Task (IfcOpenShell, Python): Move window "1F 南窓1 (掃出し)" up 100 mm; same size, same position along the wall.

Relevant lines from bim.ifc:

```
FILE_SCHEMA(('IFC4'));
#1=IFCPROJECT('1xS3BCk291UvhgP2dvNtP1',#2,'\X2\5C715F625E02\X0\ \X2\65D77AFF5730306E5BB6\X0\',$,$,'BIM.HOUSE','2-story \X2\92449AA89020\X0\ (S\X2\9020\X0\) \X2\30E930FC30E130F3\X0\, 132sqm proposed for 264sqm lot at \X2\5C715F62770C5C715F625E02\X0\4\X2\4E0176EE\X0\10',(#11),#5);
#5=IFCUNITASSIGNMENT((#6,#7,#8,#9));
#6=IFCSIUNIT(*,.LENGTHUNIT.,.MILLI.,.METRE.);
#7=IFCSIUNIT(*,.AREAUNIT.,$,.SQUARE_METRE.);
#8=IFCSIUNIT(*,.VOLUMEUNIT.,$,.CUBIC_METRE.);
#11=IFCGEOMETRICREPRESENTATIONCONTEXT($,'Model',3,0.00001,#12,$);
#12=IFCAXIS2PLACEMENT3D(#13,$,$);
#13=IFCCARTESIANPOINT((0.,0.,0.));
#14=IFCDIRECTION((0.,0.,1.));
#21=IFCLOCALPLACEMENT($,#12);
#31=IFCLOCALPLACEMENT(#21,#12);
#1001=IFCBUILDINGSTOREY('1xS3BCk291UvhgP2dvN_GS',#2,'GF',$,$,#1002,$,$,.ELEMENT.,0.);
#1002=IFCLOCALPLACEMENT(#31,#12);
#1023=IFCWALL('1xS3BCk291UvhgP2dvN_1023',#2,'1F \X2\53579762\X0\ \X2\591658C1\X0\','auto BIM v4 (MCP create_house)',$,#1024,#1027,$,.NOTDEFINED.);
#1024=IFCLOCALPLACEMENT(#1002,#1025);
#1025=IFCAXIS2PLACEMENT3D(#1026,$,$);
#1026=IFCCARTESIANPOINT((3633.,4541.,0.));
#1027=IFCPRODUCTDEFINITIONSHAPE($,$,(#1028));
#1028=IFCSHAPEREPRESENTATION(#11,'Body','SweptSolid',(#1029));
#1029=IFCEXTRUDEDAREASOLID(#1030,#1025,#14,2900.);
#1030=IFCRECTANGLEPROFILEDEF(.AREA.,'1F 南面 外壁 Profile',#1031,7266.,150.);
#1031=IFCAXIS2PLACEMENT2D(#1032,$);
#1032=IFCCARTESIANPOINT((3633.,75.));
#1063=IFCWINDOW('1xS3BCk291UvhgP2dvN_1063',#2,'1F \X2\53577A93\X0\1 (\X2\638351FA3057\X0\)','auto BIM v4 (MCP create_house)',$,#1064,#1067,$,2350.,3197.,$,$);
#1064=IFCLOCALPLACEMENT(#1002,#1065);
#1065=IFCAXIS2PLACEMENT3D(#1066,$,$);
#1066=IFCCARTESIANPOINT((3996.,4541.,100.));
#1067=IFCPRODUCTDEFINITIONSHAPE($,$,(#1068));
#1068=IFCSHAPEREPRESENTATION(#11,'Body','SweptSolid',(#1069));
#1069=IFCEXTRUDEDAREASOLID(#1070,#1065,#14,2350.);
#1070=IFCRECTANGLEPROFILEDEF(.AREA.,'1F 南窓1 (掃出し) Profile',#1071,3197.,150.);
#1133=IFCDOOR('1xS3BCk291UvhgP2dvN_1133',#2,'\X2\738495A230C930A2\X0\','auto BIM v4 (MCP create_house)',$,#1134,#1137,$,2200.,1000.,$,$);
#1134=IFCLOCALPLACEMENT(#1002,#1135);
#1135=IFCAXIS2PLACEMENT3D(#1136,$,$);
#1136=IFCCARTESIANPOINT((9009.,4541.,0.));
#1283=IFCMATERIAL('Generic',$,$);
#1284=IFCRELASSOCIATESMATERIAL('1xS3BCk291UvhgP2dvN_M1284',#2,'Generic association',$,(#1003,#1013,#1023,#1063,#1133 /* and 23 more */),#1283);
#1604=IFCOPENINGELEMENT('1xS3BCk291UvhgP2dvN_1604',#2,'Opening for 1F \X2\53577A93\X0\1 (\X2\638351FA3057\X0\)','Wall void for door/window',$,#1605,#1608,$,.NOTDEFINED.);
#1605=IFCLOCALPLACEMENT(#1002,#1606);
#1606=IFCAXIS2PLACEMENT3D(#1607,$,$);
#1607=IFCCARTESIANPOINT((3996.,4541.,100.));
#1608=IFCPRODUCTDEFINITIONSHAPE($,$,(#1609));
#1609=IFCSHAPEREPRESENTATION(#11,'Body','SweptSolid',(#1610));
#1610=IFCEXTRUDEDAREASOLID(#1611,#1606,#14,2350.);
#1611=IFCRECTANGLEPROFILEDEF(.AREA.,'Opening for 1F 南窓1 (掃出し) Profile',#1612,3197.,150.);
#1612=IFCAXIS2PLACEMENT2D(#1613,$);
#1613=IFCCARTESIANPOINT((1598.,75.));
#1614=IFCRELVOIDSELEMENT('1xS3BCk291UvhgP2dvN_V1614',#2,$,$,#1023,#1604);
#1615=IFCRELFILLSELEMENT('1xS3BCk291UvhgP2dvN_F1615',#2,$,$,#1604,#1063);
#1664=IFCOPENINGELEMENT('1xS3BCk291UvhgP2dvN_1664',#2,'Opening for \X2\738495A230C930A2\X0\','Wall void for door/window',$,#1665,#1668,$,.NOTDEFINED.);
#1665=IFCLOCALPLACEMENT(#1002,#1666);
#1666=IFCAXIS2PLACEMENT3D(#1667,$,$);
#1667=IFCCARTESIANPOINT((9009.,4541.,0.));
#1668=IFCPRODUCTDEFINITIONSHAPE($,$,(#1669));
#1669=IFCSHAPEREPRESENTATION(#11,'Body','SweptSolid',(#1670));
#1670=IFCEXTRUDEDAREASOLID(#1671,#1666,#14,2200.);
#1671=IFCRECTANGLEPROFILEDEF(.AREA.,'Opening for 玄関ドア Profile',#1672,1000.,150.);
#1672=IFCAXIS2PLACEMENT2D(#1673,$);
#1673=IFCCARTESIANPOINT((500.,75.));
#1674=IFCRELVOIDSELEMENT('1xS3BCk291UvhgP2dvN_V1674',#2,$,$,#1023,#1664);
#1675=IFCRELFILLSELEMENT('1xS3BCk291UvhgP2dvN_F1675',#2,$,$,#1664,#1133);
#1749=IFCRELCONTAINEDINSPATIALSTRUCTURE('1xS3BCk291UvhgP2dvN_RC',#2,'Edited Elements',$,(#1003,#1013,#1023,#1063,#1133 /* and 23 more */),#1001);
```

```python
import numpy as np
import ifcopenshell
import ifcopenshell.api.geometry
import ifcopenshell.util.placement
import ifcopenshell.util.unit

model = ifcopenshell.open("bim.ifc")
unit_scale = ifcopenshell.util.unit.calculate_unit_scale(model)

window = model.by_guid("1xS3BCk291UvhgP2dvN_1063")
opening = window.FillsVoids[0].RelatingOpeningElement
dz = 100.0

shift = np.array([0.0, 0.0, dz])
# The window is not placed relative to its opening, so move both.
for product in (opening, window):
    matrix = ifcopenshell.util.placement.get_local_placement(product.ObjectPlacement)
    matrix[:3, 3] += shift
    ifcopenshell.api.geometry.edit_object_placement(model, product=product, matrix=matrix, is_si=False)

print(f"moved by {dz * unit_scale:+.3f} m")

model.write("bim_updated.ifc")
```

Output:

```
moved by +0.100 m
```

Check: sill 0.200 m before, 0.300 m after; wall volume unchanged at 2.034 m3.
